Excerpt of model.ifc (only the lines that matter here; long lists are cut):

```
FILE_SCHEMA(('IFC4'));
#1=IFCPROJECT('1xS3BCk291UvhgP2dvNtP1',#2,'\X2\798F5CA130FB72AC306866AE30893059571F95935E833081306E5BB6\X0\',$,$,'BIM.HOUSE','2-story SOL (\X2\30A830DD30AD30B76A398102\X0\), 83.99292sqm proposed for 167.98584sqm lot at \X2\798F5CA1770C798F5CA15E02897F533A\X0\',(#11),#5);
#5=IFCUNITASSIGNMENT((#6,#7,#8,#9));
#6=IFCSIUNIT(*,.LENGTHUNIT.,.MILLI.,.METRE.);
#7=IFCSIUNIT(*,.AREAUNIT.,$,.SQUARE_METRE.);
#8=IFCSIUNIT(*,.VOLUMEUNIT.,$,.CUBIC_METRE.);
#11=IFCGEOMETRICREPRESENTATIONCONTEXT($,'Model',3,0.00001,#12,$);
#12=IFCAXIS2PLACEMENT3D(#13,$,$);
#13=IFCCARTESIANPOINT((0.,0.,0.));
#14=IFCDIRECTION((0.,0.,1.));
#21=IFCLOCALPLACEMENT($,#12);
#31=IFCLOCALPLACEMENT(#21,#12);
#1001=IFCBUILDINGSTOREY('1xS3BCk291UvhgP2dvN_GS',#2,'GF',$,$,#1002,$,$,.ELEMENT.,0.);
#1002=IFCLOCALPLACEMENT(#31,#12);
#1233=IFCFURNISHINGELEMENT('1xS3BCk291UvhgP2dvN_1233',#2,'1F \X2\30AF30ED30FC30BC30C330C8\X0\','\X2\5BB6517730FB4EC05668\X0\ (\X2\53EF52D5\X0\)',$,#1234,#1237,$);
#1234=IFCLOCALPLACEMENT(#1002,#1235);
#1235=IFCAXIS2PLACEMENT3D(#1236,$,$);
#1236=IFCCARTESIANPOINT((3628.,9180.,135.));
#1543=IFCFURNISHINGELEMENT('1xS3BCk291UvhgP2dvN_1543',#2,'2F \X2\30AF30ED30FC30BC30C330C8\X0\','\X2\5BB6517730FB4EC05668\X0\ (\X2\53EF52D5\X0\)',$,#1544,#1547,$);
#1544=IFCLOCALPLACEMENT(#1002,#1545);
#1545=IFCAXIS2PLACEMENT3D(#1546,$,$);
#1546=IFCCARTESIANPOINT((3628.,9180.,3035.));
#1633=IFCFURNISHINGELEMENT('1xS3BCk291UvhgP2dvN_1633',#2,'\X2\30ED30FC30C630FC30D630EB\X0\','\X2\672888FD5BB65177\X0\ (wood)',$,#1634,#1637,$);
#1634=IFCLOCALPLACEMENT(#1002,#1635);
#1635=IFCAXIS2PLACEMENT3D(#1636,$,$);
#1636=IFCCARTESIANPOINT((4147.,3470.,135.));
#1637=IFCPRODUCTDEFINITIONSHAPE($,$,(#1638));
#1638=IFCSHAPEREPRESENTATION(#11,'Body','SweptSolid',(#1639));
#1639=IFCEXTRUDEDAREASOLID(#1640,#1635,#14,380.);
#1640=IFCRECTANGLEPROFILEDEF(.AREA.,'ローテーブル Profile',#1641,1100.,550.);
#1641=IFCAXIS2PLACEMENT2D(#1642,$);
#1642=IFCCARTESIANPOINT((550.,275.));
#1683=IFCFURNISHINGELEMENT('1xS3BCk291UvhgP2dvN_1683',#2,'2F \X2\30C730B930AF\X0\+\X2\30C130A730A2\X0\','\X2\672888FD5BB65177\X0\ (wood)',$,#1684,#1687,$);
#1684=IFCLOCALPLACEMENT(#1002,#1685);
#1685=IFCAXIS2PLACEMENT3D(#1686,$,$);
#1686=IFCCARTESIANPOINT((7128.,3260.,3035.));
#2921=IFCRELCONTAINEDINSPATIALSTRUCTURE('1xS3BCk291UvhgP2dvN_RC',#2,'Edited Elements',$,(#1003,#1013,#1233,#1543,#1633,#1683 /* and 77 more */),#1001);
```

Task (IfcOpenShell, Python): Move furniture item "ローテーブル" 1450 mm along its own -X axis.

```python
import ifcopenshell
import ifcopenshell.api.geometry
import ifcopenshell.util.placement

model = ifcopenshell.open("model.ifc")

item = model.by_id(1633)
matrix = ifcopenshell.util.placement.get_local_placement(item.ObjectPlacement)
matrix[:3, 3] -= matrix[:3, 0] * 1450.0
ifcopenshell.api.geometry.edit_object_placement(model, product=item, matrix=matrix, is_si=False)

print(ifcopenshell.util.placement.get_local_placement(item.ObjectPlacement).round(3) + 0.0)

model.write("model_v2.ifc")
```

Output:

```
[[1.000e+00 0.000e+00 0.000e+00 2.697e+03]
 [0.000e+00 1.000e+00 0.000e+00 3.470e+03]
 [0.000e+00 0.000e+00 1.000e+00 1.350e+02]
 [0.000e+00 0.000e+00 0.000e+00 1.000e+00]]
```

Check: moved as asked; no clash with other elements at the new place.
